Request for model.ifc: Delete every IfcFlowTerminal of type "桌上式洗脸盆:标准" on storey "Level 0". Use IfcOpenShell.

First a look at what the model holds.

```python
import ifcopenshell
import ifcopenshell.util.element

model = ifcopenshell.open("model.ifc")
print(model.schema)
storey = next(s for s in model.by_type("IfcBuildingStorey") if s.Name == "Level 0")
terminals = [e for e in ifcopenshell.util.element.get_decomposition(storey) if e.is_a("IfcFlowTerminal")]
seen = {}
for e in terminals:
    element_type = ifcopenshell.util.element.get_type(e)
    name = element_type.Name if element_type not in (None, e) else None
    seen[name] = seen.get(name, 0) + 1
for name, count in sorted(seen.items(), key=str):
    print(count, "x", name)
```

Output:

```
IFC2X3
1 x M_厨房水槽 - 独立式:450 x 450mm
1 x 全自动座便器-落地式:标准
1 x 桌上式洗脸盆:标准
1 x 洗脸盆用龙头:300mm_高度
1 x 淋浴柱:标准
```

```python
import ifcopenshell
import ifcopenshell.api.root
import ifcopenshell.util.element

model = ifcopenshell.open("model.ifc")

storey = next(s for s in model.by_type("IfcBuildingStorey") if s.Name == "Level 0")
terminals = [e for e in ifcopenshell.util.element.get_decomposition(storey) if e.is_a("IfcFlowTerminal")]
targets = [e for e in terminals if (t := ifcopenshell.util.element.get_type(e)) not in (None, e) and t.Name == "桌上式洗脸盆:标准"]

for e in targets:
    ifcopenshell.api.root.remove_product(model, product=e)
print(len(targets), "removed")

model.write("model_rev.ifc")
```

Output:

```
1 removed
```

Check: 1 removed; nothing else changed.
